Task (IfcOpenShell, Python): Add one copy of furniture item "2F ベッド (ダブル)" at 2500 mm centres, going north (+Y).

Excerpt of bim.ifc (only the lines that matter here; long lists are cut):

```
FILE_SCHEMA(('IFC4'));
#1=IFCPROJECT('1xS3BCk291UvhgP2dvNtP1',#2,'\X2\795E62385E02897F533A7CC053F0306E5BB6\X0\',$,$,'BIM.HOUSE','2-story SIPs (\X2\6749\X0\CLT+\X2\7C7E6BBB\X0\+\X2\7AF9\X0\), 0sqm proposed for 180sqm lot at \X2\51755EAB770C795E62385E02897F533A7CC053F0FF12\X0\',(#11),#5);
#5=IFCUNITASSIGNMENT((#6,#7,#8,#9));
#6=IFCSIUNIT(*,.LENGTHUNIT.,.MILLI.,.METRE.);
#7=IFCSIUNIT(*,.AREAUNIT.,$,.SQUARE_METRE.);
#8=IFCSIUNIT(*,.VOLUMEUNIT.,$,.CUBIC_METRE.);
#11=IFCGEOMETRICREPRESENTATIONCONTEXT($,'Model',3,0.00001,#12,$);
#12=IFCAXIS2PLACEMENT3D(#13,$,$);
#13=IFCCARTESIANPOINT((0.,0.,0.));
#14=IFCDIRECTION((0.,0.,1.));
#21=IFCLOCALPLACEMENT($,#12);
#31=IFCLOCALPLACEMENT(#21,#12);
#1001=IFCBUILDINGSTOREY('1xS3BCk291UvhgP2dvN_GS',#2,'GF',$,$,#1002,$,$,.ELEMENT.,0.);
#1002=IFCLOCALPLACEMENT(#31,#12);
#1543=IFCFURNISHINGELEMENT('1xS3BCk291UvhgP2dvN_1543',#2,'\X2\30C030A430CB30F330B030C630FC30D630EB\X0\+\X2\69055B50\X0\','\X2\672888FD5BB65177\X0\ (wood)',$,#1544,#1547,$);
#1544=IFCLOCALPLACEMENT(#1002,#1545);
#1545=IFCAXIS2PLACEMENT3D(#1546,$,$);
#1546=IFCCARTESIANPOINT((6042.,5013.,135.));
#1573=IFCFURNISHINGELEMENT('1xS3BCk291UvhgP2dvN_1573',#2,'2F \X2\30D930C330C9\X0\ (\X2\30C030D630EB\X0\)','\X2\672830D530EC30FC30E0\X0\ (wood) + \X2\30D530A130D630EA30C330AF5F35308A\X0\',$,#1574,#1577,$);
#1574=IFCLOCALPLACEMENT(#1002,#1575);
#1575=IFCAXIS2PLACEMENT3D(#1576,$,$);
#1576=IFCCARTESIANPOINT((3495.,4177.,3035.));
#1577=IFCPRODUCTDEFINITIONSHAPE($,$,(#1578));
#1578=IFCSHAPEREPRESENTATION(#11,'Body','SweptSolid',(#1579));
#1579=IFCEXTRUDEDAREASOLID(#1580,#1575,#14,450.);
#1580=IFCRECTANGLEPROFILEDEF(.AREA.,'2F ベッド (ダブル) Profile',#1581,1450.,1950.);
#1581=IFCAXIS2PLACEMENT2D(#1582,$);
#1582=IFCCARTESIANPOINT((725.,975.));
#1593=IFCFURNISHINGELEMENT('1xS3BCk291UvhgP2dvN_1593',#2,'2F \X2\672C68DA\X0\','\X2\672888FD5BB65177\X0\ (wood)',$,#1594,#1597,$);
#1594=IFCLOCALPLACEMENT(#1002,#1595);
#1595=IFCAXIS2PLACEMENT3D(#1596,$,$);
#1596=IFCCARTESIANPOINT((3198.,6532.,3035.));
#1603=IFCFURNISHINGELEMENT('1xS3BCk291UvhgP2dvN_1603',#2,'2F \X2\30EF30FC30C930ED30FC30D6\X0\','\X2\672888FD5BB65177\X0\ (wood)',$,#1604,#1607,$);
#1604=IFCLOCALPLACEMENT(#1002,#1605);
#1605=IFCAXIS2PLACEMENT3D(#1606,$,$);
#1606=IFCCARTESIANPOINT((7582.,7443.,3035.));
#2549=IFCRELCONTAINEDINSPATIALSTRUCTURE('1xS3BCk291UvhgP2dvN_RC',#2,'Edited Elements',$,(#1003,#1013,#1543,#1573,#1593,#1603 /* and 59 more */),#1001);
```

```python
import numpy as np
import ifcopenshell
import ifcopenshell.api.geometry
import ifcopenshell.api.root
import ifcopenshell.util.element
import ifcopenshell.util.placement

model = ifcopenshell.open("bim.ifc")


def reuse_history(source, copy):
    """copy_class also copies each property set's owner history, people and application; keep the originals."""
    for rel in copy.IsDefinedBy:
        if rel.is_a("IfcRelDefinesByProperties") and (history := rel.RelatingPropertyDefinition.OwnerHistory):
            rel.RelatingPropertyDefinition.OwnerHistory = source.OwnerHistory
            ifcopenshell.util.element.remove_deep2(model, history)


source = model.by_guid("1xS3BCk291UvhgP2dvN_1573")
base = ifcopenshell.util.placement.get_local_placement(source.ObjectPlacement)
step = np.array([0.0, 1.0, 0.0]) * 2500.0

for i in range(1, 2):
    copy = ifcopenshell.api.root.copy_class(model, product=source)
    copy.Representation = ifcopenshell.util.element.copy_deep(
        model, source.Representation, exclude=["IfcGeometricRepresentationContext", "IfcRepresentationMap"]
    )
    reuse_history(source, copy)
    matrix = base.copy()
    matrix[:3, 3] += i * step
    print("added at", matrix[:3, 3].round(3) + 0.0)
    ifcopenshell.api.geometry.edit_object_placement(model, product=copy, matrix=matrix, is_si=False)

model.write("bim-out.ifc")
```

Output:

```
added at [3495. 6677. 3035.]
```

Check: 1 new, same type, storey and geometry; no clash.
